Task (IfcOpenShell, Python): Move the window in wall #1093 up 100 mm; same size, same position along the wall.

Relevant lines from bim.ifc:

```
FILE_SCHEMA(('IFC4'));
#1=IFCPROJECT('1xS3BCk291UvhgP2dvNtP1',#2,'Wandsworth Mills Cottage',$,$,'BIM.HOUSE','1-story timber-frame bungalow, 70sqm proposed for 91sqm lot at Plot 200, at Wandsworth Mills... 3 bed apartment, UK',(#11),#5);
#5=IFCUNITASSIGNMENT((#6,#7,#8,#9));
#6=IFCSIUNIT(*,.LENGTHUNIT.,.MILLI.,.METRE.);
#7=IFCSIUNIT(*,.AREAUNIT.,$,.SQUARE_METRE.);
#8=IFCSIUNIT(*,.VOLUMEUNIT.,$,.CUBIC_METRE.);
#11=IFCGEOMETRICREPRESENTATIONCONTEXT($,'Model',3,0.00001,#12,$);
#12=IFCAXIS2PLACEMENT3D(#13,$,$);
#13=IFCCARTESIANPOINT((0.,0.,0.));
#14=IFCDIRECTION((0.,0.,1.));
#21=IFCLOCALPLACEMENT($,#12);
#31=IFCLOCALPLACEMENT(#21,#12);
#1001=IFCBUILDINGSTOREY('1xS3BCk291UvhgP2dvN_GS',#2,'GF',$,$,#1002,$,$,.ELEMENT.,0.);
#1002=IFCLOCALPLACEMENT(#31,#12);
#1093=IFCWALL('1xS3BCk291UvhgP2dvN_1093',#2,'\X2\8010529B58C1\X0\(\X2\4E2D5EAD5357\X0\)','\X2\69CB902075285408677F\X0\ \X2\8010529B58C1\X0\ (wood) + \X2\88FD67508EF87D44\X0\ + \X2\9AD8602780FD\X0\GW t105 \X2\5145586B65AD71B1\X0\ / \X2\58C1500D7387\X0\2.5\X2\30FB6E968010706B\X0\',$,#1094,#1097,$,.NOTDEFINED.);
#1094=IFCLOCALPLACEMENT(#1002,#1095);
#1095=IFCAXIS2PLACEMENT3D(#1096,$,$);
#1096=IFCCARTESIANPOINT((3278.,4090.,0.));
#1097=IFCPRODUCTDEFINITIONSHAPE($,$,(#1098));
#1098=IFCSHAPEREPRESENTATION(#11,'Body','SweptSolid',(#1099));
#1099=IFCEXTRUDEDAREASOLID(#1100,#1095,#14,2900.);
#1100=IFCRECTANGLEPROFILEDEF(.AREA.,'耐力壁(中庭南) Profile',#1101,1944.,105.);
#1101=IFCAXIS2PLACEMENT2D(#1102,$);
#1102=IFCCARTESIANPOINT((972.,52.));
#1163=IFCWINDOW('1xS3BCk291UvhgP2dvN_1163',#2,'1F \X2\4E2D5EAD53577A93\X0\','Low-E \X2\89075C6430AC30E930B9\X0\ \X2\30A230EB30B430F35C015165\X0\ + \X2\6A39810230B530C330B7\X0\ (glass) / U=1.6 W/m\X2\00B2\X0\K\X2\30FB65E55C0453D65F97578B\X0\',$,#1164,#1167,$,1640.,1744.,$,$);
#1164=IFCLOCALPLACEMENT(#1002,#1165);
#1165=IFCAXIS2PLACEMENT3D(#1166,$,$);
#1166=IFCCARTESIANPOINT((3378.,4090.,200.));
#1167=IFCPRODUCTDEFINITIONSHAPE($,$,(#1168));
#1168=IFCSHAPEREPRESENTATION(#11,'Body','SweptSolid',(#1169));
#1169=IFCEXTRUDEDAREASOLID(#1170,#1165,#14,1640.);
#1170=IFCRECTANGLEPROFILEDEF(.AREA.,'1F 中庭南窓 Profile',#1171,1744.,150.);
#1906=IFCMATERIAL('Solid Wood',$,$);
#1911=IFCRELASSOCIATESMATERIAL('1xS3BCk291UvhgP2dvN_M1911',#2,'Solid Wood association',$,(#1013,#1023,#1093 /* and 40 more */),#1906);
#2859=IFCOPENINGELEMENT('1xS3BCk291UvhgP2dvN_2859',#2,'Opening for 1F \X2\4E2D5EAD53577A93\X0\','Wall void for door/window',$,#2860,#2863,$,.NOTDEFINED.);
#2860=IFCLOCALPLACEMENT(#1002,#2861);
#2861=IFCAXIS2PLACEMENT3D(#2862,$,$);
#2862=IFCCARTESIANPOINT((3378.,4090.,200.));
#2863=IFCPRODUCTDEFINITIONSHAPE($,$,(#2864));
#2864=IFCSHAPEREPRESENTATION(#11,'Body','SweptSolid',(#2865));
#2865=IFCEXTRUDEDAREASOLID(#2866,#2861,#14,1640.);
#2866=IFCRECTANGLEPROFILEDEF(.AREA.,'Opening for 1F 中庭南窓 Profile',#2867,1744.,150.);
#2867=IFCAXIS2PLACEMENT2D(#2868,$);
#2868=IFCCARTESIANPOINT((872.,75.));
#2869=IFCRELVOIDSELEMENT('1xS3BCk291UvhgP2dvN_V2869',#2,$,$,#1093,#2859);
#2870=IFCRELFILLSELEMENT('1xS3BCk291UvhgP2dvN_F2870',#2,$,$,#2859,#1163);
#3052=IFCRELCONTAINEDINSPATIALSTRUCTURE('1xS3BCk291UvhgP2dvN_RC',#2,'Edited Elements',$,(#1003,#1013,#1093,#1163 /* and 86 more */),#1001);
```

```python
import numpy as np
import ifcopenshell
import ifcopenshell.api.geometry
import ifcopenshell.util.placement
import ifcopenshell.util.unit

model = ifcopenshell.open("bim.ifc")
unit_scale = ifcopenshell.util.unit.calculate_unit_scale(model)

window = model.by_guid("1xS3BCk291UvhgP2dvN_1163")
opening = window.FillsVoids[0].RelatingOpeningElement
dz = 0.1 / unit_scale

shift = np.array([0.0, 0.0, dz])
# The window is not placed relative to its opening, so move both.
for product in (opening, window):
    matrix = ifcopenshell.util.placement.get_local_placement(product.ObjectPlacement)
    matrix[:3, 3] += shift
    ifcopenshell.api.geometry.edit_object_placement(model, product=product, matrix=matrix, is_si=False)

print(f"moved by {dz * unit_scale:+.3f} m")

model.write("bim_edited.ifc")
```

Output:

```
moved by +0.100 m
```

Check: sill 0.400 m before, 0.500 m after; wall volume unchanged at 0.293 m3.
